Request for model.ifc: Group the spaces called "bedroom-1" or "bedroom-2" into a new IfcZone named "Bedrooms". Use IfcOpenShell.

First a look at what the model holds.

```python
import ifcopenshell

model = ifcopenshell.open("model.ifc")
print(model.schema)
seen = {}
for space in model.by_type("IfcSpace"):
    seen[space.Name] = seen.get(space.Name, 0) + 1
for name, count in sorted(seen.items(), key=str):
    print(count, "x", name)
print("zones:", [z.Name for z in model.by_type("IfcZone")][:20])
```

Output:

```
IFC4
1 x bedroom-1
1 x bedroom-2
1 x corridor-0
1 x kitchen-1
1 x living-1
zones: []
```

```python
import ifcopenshell
import ifcopenshell.api.group
import ifcopenshell.api.root

model = ifcopenshell.open("model.ifc")

names = {"bedroom-1", "bedroom-2"}
spaces = [s for s in model.by_type("IfcSpace") if s.Name in names]

zone = ifcopenshell.api.root.create_entity(model, ifc_class="IfcZone", name="Bedrooms")
ifcopenshell.api.group.assign_group(model, products=spaces, group=zone)
print(len(spaces), "spaces in", zone.Name)

model.write("model_edited.ifc")
```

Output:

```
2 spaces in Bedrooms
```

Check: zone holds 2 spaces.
